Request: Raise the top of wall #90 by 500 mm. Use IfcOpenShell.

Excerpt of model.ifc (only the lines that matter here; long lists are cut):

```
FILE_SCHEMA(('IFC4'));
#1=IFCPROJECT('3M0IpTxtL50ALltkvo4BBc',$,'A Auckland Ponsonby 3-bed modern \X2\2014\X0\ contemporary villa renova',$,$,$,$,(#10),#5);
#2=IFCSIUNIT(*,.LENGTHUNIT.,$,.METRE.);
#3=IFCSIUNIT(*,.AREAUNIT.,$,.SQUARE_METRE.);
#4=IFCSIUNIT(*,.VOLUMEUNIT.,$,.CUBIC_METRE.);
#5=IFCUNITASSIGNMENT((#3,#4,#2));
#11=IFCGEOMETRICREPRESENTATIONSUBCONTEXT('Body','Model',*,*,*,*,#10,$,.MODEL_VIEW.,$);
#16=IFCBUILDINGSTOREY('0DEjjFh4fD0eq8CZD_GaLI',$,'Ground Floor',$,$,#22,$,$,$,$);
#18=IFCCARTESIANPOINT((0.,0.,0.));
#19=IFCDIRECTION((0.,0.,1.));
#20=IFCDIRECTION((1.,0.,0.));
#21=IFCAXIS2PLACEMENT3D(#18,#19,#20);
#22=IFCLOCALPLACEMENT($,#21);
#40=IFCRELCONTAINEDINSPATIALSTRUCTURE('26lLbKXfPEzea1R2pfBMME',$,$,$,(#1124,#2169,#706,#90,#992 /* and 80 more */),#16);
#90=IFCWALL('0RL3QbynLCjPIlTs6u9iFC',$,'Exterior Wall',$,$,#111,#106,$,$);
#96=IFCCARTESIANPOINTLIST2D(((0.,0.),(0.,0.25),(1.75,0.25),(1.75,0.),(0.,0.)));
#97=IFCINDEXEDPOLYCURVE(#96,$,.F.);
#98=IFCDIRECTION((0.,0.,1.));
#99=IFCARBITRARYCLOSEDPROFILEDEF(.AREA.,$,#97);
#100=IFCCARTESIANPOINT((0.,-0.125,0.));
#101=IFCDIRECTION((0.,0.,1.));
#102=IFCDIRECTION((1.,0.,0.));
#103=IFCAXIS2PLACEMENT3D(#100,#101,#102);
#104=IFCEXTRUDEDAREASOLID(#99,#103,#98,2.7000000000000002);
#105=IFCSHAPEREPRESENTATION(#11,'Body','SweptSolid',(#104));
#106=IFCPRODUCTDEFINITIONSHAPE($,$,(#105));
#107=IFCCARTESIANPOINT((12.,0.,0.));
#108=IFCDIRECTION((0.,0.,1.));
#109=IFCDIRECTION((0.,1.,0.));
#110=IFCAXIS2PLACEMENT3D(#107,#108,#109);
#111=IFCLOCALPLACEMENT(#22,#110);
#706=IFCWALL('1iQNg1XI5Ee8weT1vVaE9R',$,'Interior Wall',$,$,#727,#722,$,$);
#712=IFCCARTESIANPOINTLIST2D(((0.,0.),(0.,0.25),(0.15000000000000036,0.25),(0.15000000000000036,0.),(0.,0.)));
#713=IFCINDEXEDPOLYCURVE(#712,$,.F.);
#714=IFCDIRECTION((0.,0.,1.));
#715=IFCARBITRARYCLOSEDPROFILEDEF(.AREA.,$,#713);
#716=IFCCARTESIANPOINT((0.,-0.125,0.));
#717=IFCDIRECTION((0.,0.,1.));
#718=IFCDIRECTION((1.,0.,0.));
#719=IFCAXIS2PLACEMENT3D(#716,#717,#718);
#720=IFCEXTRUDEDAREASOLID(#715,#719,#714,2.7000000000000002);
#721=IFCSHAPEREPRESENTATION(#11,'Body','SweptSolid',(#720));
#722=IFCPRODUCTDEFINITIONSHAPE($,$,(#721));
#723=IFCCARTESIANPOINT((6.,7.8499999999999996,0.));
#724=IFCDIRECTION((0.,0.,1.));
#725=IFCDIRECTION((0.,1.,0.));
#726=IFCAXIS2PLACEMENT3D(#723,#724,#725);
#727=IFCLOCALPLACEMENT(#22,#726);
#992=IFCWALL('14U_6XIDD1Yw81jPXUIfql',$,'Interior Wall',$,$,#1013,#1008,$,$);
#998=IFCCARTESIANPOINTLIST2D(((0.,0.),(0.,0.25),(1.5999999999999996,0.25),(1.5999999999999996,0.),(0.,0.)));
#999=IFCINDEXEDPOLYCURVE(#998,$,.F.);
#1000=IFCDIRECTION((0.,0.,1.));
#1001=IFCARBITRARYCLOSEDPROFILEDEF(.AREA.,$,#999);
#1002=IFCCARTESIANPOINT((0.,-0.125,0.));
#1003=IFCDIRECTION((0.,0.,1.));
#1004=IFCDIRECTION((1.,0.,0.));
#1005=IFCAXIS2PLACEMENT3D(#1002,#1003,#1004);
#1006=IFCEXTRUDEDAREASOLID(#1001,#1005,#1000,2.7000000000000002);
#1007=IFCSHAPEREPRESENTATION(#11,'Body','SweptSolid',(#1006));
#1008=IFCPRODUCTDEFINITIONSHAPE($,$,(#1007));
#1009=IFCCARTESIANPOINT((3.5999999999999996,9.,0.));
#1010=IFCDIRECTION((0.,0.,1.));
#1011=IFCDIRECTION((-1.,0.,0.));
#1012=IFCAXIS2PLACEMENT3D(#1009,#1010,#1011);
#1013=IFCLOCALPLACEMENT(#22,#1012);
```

```python
import ifcopenshell
import ifcopenshell.geom
import ifcopenshell.util.representation
import ifcopenshell.util.shape
import ifcopenshell.util.unit

model = ifcopenshell.open("model.ifc")
unit_scale = ifcopenshell.util.unit.calculate_unit_scale(model)
settings = ifcopenshell.geom.settings()


def volume(element):
    """Net volume in cubic metres, openings subtracted."""
    shape = ifcopenshell.geom.create_shape(settings, element)
    return ifcopenshell.util.shape.get_volume(shape.geometry)


wall = model.by_guid("0RL3QbynLCjPIlTs6u9iFC")
before = volume(wall)

body = ifcopenshell.util.representation.get_representation(wall, "Model", "Body")
solid = body.Items[0]
old_height = solid.Depth
solid.Depth += 0.5 / unit_scale
after = volume(wall)

print(f"height {old_height:g} -> {solid.Depth:g}, volume {before:.3f} -> {after:.3f} m3")

model.write("model-out.ifc")
```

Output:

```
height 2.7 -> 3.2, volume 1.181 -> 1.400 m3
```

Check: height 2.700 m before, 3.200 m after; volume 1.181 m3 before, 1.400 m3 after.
